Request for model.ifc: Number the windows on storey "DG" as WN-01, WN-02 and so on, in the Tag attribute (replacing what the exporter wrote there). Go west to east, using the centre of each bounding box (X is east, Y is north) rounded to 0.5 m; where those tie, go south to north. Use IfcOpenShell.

First a look at what the model holds.

```python
import ifcopenshell
import ifcopenshell.util.element
import ifcopenshell.util.placement

model = ifcopenshell.open("model.ifc")
print(model.schema)
storey = next(s for s in model.by_type("IfcBuildingStorey") if s.Name == "DG")
windows = [e for e in ifcopenshell.util.element.get_decomposition(storey) if e.is_a("IfcWindow")]
for e in sorted(windows, key=lambda e: e.id()):
    origin = ifcopenshell.util.placement.get_local_placement(e.ObjectPlacement)[:3, 3]
    print(e.id(), e.Tag, e.Name, origin.round(2) + 0.0, sep=" | ")
```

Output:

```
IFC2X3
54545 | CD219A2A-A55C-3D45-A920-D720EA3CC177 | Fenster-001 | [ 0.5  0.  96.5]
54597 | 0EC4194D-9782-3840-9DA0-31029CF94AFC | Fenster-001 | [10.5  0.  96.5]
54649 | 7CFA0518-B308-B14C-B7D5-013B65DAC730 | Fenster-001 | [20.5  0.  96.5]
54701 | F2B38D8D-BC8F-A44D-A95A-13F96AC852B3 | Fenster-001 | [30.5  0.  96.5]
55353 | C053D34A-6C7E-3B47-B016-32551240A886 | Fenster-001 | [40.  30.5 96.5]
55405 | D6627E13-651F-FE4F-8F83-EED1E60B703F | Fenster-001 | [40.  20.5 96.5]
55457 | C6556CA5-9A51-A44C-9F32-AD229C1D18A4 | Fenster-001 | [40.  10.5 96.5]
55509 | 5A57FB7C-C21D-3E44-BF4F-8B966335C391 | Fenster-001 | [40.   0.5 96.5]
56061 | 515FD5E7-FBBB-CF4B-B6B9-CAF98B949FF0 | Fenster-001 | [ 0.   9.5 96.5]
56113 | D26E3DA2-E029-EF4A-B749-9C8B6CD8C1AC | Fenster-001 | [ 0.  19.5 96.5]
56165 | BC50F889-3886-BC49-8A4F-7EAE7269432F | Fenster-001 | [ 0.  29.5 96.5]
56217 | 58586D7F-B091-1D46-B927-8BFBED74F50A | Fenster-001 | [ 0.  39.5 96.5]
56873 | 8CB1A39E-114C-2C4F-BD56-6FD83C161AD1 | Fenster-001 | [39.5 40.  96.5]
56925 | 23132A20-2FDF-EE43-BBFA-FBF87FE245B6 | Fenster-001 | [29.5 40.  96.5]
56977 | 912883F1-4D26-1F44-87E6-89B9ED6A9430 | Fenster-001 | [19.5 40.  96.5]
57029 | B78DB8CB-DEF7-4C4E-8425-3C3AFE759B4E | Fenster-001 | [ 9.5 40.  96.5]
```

```python
import ifcopenshell
import ifcopenshell.geom
import ifcopenshell.util.element
import ifcopenshell.util.shape

model = ifcopenshell.open("model.ifc")
settings = ifcopenshell.geom.settings()
settings.set("use-world-coords", True)


def centre(element):
    shape = ifcopenshell.geom.create_shape(settings, element)
    return ifcopenshell.util.shape.get_bbox_centroid(shape.geometry)


storey = next(s for s in model.by_type("IfcBuildingStorey") if s.Name == "DG")
windows = [e for e in ifcopenshell.util.element.get_decomposition(storey) if e.is_a("IfcWindow")]

# Insertion points can sit at a corner or the storey origin, so sort by the geometry (in metres).
centres = {e: centre(e) for e in windows}
windows.sort(key=lambda e: (round(centres[e][0] / 0.5), centres[e][1]))

for i, e in enumerate(windows, start=1):
    number = f"WN-{i:02d}"
    e.Tag = number
    print(e.id(), number)

model.write("model_edited.ifc")
```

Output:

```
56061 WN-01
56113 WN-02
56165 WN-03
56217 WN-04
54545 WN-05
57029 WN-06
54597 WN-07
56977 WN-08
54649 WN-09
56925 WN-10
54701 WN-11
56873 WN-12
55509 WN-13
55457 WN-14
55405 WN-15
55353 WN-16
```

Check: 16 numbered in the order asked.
